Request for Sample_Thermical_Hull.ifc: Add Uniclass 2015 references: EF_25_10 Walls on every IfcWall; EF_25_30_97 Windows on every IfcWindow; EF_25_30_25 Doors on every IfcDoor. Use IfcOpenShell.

First a look at what the model holds.

```python
import ifcopenshell

model = ifcopenshell.open("Sample_Thermical_Hull.ifc")
print(model.schema)
print("classifications:", [c.Name for c in model.by_type("IfcClassification")])
for ifc_class in ("IfcDoor", "IfcRoof", "IfcStair", "IfcWall", "IfcWindow"):
    print(ifc_class, len(model.by_type(ifc_class)))
```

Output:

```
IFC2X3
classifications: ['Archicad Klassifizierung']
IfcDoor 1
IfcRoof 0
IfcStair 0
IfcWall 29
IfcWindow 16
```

```python
import ifcopenshell
import ifcopenshell.api.classification

model = ifcopenshell.open("Sample_Thermical_Hull.ifc")

# IFC2X3 requires Source and Edition and has no link from the project to the system.
system = model.create_entity("IfcClassification", Source="NBS", Edition="2015", Name="Uniclass 2015")

codes = {
    "IfcWall": ("EF_25_10", "Walls"),
    "IfcWindow": ("EF_25_30_97", "Windows"),
    "IfcDoor": ("EF_25_30_25", "Doors"),
}
for ifc_class, (code, name) in codes.items():
    products = model.by_type(ifc_class)
    ifcopenshell.api.classification.add_reference(
        model, products=products, classification=system, identification=code, name=name
    )
    print(code, len(products))

model.write("Sample_Thermical_Hull_rev.ifc")
```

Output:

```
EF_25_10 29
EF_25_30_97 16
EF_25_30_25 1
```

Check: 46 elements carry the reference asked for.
